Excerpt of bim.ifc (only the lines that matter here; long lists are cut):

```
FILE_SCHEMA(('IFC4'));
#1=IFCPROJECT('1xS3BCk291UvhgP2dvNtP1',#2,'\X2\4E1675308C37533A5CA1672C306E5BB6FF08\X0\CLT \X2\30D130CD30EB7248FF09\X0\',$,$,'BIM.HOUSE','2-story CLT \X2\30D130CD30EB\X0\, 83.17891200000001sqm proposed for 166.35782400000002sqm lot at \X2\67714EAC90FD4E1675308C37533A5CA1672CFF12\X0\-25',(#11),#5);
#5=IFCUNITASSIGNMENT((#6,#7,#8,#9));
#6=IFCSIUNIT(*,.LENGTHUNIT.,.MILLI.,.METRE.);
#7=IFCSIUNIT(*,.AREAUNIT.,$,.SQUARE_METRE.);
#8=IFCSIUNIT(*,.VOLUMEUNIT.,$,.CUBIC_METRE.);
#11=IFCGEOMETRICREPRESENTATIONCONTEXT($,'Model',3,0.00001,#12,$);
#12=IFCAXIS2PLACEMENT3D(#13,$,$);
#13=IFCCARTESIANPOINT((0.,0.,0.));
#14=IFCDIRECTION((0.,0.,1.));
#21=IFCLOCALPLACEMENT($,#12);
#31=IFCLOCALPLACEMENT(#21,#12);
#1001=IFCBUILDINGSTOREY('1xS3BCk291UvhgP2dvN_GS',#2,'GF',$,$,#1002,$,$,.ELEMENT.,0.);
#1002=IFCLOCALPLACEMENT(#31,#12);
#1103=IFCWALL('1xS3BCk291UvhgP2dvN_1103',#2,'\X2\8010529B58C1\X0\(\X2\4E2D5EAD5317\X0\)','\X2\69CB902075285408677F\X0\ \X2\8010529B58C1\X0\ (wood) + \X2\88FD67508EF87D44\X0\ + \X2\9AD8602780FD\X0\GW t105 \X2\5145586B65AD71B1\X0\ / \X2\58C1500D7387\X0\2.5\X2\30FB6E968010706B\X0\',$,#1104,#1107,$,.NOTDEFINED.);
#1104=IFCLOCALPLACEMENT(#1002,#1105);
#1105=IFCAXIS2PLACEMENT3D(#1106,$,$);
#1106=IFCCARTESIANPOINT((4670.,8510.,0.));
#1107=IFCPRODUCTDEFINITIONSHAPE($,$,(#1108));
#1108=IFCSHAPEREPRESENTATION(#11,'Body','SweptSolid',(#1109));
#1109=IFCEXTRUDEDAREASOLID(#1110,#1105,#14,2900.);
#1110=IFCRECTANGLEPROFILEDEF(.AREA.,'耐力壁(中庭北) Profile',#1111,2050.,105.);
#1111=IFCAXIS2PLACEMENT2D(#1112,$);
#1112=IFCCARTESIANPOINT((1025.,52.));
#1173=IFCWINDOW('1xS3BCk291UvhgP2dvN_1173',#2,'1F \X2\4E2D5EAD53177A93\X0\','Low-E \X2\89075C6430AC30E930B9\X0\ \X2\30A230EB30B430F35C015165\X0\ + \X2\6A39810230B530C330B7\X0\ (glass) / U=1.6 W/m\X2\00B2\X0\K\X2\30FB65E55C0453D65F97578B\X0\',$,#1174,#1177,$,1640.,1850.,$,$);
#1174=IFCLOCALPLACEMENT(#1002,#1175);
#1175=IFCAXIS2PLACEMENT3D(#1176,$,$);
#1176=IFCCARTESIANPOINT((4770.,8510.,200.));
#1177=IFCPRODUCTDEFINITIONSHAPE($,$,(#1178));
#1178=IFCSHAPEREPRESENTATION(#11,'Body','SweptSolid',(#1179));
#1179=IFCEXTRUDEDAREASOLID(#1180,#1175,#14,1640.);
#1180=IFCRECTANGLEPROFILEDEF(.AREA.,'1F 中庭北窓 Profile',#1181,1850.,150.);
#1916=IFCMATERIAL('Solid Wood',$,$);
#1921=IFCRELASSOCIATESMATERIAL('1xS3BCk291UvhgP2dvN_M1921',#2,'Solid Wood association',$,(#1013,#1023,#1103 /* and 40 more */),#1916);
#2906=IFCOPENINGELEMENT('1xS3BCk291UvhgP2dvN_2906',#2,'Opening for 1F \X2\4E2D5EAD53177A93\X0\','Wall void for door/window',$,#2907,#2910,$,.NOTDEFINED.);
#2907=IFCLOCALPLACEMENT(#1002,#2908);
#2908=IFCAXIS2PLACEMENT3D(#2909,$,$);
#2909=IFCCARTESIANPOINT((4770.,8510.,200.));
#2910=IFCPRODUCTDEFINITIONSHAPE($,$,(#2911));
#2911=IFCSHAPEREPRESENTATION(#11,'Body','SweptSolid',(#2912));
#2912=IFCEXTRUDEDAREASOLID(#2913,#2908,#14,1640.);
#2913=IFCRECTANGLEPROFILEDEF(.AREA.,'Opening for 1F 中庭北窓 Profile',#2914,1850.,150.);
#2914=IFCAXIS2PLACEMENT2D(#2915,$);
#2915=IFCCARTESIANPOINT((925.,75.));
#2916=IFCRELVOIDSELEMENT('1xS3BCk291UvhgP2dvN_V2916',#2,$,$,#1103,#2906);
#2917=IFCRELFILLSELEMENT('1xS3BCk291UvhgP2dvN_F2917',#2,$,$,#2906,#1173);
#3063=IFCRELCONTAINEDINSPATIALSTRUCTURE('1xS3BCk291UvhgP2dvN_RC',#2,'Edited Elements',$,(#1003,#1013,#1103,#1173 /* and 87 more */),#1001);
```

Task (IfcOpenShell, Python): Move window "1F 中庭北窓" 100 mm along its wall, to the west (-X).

```python
import ifcopenshell
import ifcopenshell.api.geometry
import ifcopenshell.util.placement
import ifcopenshell.util.unit

model = ifcopenshell.open("bim.ifc")
unit_scale = ifcopenshell.util.unit.calculate_unit_scale(model)

window = model.by_guid("1xS3BCk291UvhgP2dvN_1173")
opening = window.FillsVoids[0].RelatingOpeningElement
wall = opening.VoidsElements[0].RelatingBuildingElement

wall_matrix = ifcopenshell.util.placement.get_local_placement(wall.ObjectPlacement)
shift = wall_matrix[:3, 0] * -0.1 / unit_scale
before = ifcopenshell.util.placement.get_local_placement(window.ObjectPlacement)[:3, 3].copy()

# The window is not placed relative to its opening, so move both.
for product in (opening, window):
    matrix = ifcopenshell.util.placement.get_local_placement(product.ObjectPlacement)
    matrix[:3, 3] += shift
    ifcopenshell.api.geometry.edit_object_placement(model, product=product, matrix=matrix, is_si=False)

after = ifcopenshell.util.placement.get_local_placement(window.ObjectPlacement)[:3, 3]
print("window moved by", (after - before).round(3) + 0.0)

model.write("bim-out.ifc")
```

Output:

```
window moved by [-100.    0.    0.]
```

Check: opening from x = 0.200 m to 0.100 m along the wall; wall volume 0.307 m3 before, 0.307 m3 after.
